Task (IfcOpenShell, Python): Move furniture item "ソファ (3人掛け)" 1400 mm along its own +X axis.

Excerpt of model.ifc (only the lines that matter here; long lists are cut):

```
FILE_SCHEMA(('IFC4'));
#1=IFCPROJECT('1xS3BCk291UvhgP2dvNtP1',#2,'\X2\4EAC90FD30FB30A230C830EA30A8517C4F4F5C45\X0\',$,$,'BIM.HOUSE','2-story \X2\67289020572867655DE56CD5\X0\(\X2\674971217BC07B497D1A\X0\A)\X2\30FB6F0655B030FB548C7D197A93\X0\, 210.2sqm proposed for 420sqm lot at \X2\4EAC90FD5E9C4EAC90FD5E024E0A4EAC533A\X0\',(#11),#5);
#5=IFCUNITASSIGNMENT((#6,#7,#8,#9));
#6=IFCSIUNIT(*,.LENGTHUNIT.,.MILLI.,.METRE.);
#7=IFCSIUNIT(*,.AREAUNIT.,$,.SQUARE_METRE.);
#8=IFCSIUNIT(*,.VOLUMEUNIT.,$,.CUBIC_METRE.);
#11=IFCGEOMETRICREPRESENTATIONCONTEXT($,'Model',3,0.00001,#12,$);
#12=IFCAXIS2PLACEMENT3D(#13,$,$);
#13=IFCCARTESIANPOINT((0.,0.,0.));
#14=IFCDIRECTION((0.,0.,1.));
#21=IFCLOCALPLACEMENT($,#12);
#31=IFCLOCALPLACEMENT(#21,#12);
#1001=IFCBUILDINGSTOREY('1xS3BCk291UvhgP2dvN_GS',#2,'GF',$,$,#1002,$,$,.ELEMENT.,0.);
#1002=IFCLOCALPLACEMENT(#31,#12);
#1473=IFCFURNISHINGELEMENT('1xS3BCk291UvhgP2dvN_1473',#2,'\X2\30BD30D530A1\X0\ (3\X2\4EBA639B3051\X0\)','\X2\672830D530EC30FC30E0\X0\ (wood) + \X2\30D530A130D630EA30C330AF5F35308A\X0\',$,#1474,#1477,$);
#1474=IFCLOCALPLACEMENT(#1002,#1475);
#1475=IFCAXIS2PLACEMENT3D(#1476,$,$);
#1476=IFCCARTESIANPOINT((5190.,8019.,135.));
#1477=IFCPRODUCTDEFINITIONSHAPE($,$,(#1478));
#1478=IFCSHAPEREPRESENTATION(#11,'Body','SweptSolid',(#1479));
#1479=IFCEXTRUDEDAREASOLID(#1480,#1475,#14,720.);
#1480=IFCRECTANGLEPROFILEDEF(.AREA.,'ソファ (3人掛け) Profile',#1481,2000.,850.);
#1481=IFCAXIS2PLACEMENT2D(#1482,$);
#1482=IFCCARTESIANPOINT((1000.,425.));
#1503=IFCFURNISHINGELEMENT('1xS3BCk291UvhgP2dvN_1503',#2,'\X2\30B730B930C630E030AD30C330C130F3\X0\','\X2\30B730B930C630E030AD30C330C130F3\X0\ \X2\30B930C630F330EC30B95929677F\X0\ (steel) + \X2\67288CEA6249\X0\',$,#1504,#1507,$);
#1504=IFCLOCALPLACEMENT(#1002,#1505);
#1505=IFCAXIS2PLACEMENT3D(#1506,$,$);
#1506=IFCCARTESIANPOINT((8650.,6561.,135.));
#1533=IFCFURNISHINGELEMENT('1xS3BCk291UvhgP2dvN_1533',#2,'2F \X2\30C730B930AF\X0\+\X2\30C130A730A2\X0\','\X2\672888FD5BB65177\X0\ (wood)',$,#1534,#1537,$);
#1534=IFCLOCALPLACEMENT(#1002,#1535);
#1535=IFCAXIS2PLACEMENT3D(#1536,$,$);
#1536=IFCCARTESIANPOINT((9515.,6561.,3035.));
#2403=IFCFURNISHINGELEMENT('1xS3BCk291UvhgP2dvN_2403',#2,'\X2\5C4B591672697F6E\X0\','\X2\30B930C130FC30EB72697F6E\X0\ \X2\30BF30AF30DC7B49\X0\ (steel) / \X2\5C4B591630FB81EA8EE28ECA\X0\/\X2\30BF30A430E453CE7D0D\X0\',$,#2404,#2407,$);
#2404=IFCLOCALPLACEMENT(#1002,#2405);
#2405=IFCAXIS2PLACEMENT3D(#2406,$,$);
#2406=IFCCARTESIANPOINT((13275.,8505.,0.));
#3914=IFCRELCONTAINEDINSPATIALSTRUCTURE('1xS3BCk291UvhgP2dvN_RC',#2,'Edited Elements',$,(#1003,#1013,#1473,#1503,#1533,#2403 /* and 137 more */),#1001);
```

```python
import ifcopenshell
import ifcopenshell.api.geometry
import ifcopenshell.util.placement
import ifcopenshell.util.unit

model = ifcopenshell.open("model.ifc")
unit_scale = ifcopenshell.util.unit.calculate_unit_scale(model)

item = model.by_guid("1xS3BCk291UvhgP2dvN_1473")
matrix = ifcopenshell.util.placement.get_local_placement(item.ObjectPlacement)
matrix[:3, 3] += matrix[:3, 0] * 1.4 / unit_scale
ifcopenshell.api.geometry.edit_object_placement(model, product=item, matrix=matrix, is_si=False)

print(ifcopenshell.util.placement.get_local_placement(item.ObjectPlacement).round(3) + 0.0)

model.write("model_updated.ifc")
```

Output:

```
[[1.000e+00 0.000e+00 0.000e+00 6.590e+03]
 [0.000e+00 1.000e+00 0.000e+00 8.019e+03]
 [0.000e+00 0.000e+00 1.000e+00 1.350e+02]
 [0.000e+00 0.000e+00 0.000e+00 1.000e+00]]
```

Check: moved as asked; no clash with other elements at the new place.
